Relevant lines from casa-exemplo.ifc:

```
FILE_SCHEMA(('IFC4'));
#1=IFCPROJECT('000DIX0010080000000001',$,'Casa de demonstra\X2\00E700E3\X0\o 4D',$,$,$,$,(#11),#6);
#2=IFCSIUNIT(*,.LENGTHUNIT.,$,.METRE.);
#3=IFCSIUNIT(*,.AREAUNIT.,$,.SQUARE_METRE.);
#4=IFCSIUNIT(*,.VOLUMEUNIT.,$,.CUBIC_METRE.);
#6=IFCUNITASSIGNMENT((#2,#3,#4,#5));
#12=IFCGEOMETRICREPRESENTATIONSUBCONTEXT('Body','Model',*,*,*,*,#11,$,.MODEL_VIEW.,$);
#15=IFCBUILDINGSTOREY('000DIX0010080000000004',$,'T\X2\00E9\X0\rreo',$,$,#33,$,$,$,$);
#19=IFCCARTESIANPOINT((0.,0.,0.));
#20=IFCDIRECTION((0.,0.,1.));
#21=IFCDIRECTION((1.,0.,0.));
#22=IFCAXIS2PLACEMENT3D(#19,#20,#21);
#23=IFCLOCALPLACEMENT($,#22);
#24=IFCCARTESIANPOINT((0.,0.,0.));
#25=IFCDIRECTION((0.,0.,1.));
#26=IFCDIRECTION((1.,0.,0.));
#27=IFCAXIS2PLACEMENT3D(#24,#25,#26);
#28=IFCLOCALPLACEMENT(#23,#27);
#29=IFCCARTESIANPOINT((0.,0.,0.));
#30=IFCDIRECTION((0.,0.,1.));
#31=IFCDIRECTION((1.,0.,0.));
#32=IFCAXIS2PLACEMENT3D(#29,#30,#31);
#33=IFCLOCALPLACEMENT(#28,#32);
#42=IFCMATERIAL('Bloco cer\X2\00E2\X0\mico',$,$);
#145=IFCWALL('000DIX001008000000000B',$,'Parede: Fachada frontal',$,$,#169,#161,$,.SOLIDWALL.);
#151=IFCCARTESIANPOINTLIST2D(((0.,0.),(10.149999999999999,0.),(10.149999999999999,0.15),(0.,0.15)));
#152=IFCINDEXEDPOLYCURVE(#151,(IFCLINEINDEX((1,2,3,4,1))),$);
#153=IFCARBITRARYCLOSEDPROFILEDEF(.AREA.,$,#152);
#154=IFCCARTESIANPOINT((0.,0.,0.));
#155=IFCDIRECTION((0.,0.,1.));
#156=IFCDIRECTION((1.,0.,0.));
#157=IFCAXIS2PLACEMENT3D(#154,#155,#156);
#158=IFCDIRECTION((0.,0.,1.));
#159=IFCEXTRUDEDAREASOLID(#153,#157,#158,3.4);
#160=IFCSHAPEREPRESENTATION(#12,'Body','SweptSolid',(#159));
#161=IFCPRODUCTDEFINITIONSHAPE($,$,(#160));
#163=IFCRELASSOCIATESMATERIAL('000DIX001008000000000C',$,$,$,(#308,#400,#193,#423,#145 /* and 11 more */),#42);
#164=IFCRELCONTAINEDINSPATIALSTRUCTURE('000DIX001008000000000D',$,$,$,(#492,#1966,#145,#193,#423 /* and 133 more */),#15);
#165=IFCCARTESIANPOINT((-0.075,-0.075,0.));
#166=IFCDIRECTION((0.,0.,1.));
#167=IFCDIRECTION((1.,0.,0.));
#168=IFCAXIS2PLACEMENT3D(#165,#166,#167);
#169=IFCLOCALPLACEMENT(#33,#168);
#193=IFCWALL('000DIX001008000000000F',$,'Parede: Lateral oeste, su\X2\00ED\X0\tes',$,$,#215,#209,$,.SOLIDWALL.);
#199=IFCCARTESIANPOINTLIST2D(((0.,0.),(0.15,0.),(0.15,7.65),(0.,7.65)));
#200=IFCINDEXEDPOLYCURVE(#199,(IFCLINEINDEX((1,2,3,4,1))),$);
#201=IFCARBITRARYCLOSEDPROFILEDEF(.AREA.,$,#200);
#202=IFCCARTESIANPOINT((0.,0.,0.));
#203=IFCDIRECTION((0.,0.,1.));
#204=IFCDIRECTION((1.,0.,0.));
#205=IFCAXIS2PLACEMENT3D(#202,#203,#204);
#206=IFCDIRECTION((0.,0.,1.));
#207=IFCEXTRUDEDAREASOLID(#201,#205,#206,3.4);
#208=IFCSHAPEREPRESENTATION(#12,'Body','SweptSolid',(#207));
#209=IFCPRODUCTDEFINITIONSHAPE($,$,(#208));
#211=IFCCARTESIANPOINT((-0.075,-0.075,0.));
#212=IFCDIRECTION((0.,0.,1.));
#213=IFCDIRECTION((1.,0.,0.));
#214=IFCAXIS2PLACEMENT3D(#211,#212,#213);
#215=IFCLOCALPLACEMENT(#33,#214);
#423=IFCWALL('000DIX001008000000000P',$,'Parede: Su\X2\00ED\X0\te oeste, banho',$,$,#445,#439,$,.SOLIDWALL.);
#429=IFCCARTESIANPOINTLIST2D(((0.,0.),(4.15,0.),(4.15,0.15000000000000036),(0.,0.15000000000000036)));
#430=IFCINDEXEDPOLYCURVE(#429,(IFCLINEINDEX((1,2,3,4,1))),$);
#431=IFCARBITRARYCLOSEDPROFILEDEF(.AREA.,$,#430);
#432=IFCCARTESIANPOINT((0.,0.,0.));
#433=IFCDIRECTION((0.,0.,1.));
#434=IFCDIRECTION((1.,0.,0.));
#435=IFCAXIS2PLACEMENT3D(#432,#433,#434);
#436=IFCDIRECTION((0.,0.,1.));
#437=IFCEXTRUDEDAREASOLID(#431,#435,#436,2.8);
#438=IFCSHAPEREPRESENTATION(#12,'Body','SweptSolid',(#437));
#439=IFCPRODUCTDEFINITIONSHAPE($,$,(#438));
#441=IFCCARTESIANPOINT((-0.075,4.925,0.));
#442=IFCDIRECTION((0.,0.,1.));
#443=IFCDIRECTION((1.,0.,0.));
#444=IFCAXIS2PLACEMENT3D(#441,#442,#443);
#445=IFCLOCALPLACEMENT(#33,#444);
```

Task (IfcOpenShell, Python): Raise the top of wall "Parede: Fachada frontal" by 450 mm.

```python
import ifcopenshell
import ifcopenshell.geom
import ifcopenshell.util.representation
import ifcopenshell.util.shape

model = ifcopenshell.open("casa-exemplo.ifc")
settings = ifcopenshell.geom.settings()


def volume(element):
    """Net volume in cubic metres, openings subtracted."""
    shape = ifcopenshell.geom.create_shape(settings, element)
    return ifcopenshell.util.shape.get_volume(shape.geometry)


wall = model.by_id(145)
before = volume(wall)

body = ifcopenshell.util.representation.get_representation(wall, "Model", "Body")
solid = body.Items[0]
old_height = solid.Depth
solid.Depth += 0.45
after = volume(wall)

print(f"height {old_height:g} -> {solid.Depth:g}, volume {before:.3f} -> {after:.3f} m3")

model.write("casa-exemplo-out.ifc")
```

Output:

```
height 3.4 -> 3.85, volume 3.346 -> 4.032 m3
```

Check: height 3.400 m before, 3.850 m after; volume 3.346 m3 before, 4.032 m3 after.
